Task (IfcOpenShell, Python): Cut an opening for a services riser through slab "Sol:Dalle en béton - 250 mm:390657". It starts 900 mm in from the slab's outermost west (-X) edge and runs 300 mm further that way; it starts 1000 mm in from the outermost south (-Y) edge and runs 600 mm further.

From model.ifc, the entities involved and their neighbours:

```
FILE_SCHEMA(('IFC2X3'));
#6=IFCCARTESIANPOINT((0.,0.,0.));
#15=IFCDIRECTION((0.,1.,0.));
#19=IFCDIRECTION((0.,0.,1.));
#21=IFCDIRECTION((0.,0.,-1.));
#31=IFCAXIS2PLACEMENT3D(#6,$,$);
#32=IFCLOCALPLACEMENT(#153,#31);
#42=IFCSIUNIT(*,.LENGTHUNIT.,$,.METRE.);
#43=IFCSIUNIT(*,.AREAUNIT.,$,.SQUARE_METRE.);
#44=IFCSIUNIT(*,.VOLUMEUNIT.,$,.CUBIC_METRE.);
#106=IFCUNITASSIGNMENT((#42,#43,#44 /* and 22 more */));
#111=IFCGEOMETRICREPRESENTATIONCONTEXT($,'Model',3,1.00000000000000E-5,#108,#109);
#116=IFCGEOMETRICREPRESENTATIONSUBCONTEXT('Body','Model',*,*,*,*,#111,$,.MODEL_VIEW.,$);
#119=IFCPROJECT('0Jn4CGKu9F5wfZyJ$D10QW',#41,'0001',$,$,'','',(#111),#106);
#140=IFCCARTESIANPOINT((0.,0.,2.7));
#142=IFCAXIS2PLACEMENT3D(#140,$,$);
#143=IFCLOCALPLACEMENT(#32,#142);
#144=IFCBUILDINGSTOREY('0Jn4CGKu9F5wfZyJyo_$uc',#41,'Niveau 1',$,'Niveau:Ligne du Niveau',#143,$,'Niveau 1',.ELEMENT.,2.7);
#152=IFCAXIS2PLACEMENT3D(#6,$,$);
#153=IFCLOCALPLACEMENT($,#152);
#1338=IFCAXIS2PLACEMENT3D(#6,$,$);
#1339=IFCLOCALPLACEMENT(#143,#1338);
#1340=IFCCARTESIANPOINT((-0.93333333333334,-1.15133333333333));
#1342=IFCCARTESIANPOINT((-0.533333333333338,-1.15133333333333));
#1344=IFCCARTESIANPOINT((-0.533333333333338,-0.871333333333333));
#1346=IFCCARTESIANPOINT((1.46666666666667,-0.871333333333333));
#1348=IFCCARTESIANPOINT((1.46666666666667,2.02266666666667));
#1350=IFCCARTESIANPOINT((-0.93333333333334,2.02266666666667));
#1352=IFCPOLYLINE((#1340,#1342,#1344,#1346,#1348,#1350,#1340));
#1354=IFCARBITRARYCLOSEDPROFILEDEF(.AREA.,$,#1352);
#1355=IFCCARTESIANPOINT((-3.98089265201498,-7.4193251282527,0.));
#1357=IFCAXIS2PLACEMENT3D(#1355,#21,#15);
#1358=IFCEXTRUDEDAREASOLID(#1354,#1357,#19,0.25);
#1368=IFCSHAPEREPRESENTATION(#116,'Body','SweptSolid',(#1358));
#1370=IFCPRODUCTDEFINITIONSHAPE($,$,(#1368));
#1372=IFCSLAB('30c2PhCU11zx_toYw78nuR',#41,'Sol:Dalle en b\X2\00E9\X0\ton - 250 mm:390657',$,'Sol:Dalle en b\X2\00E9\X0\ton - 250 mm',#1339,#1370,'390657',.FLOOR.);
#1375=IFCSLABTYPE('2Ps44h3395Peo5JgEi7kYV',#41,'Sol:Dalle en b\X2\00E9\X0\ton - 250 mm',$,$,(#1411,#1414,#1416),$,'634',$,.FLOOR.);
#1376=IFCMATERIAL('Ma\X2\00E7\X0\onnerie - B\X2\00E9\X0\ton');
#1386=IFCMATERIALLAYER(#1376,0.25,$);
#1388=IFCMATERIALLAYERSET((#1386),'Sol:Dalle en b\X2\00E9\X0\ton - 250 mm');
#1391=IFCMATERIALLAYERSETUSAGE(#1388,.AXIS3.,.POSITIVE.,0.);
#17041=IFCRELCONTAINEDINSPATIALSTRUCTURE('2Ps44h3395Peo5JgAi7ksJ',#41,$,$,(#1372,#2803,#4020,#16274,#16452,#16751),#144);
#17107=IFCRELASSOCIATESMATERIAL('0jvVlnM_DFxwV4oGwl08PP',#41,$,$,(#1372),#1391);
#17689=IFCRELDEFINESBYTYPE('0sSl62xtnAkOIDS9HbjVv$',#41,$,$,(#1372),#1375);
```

```python
import numpy as np
import ifcopenshell
import ifcopenshell.api.feature
import ifcopenshell.api.geometry
import ifcopenshell.api.root
import ifcopenshell.geom
import ifcopenshell.util.placement
import ifcopenshell.util.representation
import ifcopenshell.util.shape
import ifcopenshell.util.unit

model = ifcopenshell.open("model.ifc")
unit_scale = ifcopenshell.util.unit.calculate_unit_scale(model)
settings = ifcopenshell.geom.settings()


def volume(element):
    """Net volume in cubic metres, openings subtracted."""
    shape = ifcopenshell.geom.create_shape(settings, element)
    return ifcopenshell.util.shape.get_volume(shape.geometry)


slab = model.by_guid("30c2PhCU11zx_toYw78nuR")
before = volume(slab)

# Extent in the slab's own axes, in metres. The edges named are its -X and -Y sides.
slab_shape = ifcopenshell.geom.create_shape(settings, slab)
vertices = ifcopenshell.util.shape.get_vertices(slab_shape.geometry)
x_min, y_min, bottom = vertices.min(axis=0)
top = vertices[:, 2].max()

opening = ifcopenshell.api.root.create_entity(model, ifc_class="IfcOpeningElement", name="Services riser opening")
context = ifcopenshell.util.representation.get_context(model, "Model", "Body", "MODEL_VIEW")
width, depth = 0.3, 0.6
outline = [(0.0, 0.0), (width, 0.0), (width, depth), (0.0, depth), (0.0, 0.0)]
# Overshoot both faces by 50 mm so the cut is clean.
shape = ifcopenshell.api.geometry.add_slab_representation(
    model, context=context, depth=top - bottom + 0.1, polyline=outline
)
ifcopenshell.api.geometry.assign_representation(model, product=opening, representation=shape)

matrix = ifcopenshell.util.placement.get_local_placement(slab.ObjectPlacement)
matrix[:, 3] = matrix @ np.append(np.array([x_min + 0.9, y_min + 1, bottom - 0.05]) / unit_scale, 1.0)
ifcopenshell.api.geometry.edit_object_placement(model, product=opening, matrix=matrix, is_si=False)
ifcopenshell.api.feature.add_feature(model, feature=opening, element=slab)

after = volume(slab)

print(f"slab volume {before:.3f} -> {after:.3f} m3")

model.write("model_edited.ifc")
```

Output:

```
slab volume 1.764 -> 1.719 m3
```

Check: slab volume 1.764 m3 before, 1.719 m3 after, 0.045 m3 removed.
